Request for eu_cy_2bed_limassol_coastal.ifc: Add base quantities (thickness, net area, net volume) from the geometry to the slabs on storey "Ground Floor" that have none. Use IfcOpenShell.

First a look at what the model holds.

```python
import ifcopenshell
import ifcopenshell.util.element
import ifcopenshell.util.unit

model = ifcopenshell.open("eu_cy_2bed_limassol_coastal.ifc")
print(model.schema)
for unit_type in ("LENGTHUNIT", "AREAUNIT", "VOLUMEUNIT"):
    print(unit_type, ifcopenshell.util.unit.calculate_unit_scale(model, unit_type))
storey = next(s for s in model.by_type("IfcBuildingStorey") if s.Name == "Ground Floor")
slabs = [e for e in ifcopenshell.util.element.get_decomposition(storey) if e.is_a("IfcSlab")]
for e in sorted(slabs, key=lambda e: e.id()):
    print(e.id(), e.is_a(), e.Name, list(ifcopenshell.util.element.get_psets(e, qtos_only=True)), sep=" | ")
```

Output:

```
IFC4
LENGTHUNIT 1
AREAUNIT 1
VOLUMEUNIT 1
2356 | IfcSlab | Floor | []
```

```python
import ifcopenshell
import ifcopenshell.api.pset
import ifcopenshell.geom
import ifcopenshell.util.element
import ifcopenshell.util.shape
import ifcopenshell.util.unit

model = ifcopenshell.open("eu_cy_2bed_limassol_coastal.ifc")
unit_scale = ifcopenshell.util.unit.calculate_unit_scale(model)
area_scale = ifcopenshell.util.unit.calculate_unit_scale(model, "AREAUNIT")
volume_scale = ifcopenshell.util.unit.calculate_unit_scale(model, "VOLUMEUNIT")
settings = ifcopenshell.geom.settings()

storey = next(s for s in model.by_type("IfcBuildingStorey") if s.Name == "Ground Floor")
slabs = [e for e in ifcopenshell.util.element.get_decomposition(storey) if e.is_a("IfcSlab")]

for e in sorted(slabs, key=lambda e: e.id()):
    if ifcopenshell.util.element.get_psets(e, qtos_only=True, should_inherit=False):
        continue
    # Geometry comes back in metres, in the element's own axes.
    shape = ifcopenshell.geom.create_shape(settings, e)
    values = {
        "Width": ifcopenshell.util.shape.get_z(shape.geometry) / unit_scale,
        "NetArea": ifcopenshell.util.shape.get_footprint_area(shape.geometry) / area_scale,
        "NetVolume": ifcopenshell.util.shape.get_volume(shape.geometry) / volume_scale,
    }
    qto = ifcopenshell.api.pset.add_qto(model, product=e, name="Qto_SlabBaseQuantities")
    ifcopenshell.api.pset.edit_qto(model, qto=qto, properties=values)
    print(e.id(), {k: round(v, 3) for k, v in values.items()})

model.write("eu_cy_2bed_limassol_coastal_edited.ifc")
```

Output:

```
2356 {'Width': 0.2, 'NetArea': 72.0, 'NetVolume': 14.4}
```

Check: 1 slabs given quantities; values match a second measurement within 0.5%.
